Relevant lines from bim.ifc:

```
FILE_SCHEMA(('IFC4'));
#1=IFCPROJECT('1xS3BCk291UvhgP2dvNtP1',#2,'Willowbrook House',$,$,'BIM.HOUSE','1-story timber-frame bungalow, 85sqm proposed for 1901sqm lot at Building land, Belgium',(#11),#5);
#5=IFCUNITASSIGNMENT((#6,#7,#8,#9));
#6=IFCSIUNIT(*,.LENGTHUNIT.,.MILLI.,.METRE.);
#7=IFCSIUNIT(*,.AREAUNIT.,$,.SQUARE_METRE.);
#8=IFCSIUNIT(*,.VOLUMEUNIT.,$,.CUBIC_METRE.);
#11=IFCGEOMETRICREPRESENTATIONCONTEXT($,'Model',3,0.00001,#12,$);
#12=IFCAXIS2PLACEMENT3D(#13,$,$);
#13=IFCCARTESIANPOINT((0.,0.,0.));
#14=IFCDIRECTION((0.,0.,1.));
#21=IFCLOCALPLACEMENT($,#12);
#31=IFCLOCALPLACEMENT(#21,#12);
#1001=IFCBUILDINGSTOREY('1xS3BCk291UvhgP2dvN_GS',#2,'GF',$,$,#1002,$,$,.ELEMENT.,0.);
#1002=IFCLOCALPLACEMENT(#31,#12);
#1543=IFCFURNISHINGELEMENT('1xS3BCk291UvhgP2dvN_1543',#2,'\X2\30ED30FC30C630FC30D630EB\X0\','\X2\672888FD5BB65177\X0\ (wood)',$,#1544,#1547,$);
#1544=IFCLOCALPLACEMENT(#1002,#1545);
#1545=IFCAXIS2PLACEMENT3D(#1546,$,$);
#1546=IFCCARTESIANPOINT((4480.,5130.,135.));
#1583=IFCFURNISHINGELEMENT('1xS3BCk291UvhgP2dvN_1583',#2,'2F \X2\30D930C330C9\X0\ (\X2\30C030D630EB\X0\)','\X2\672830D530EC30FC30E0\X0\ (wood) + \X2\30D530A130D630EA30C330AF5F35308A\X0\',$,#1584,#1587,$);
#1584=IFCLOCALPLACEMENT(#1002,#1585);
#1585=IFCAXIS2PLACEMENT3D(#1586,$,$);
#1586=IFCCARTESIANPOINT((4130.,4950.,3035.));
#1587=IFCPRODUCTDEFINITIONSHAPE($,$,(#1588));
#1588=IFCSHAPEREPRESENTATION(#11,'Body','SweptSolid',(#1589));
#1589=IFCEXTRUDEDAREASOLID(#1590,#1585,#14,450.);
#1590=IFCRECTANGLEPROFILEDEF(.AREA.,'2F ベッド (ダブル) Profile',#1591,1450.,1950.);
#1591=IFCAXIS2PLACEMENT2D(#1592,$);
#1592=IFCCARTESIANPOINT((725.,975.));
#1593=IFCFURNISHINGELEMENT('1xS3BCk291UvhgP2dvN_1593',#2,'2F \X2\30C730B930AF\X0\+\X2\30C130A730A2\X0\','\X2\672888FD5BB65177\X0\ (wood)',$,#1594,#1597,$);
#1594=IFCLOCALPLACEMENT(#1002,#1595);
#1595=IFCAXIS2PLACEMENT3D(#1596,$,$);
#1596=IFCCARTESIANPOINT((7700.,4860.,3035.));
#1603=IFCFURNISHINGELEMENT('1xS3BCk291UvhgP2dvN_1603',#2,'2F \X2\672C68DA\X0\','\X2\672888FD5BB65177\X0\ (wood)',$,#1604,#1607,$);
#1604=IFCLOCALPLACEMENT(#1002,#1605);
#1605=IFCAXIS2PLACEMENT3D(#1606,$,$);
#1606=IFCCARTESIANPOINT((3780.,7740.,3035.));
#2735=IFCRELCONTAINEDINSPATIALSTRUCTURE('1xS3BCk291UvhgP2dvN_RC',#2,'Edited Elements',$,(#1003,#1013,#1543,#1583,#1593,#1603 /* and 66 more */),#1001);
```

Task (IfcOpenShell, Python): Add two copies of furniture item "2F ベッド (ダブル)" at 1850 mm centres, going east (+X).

```python
import numpy as np
import ifcopenshell
import ifcopenshell.api.geometry
import ifcopenshell.api.root
import ifcopenshell.util.element
import ifcopenshell.util.placement

model = ifcopenshell.open("bim.ifc")


def reuse_history(source, copy):
    """copy_class also copies each property set's owner history, people and application; keep the originals."""
    for rel in copy.IsDefinedBy:
        if rel.is_a("IfcRelDefinesByProperties") and (history := rel.RelatingPropertyDefinition.OwnerHistory):
            rel.RelatingPropertyDefinition.OwnerHistory = source.OwnerHistory
            ifcopenshell.util.element.remove_deep2(model, history)


source = model.by_guid("1xS3BCk291UvhgP2dvN_1583")
base = ifcopenshell.util.placement.get_local_placement(source.ObjectPlacement)
step = np.array([1.0, 0.0, 0.0]) * 1850.0

for i in range(1, 3):
    copy = ifcopenshell.api.root.copy_class(model, product=source)
    copy.Representation = ifcopenshell.util.element.copy_deep(
        model, source.Representation, exclude=["IfcGeometricRepresentationContext", "IfcRepresentationMap"]
    )
    reuse_history(source, copy)
    matrix = base.copy()
    matrix[:3, 3] += i * step
    print("added at", matrix[:3, 3].round(3) + 0.0)
    ifcopenshell.api.geometry.edit_object_placement(model, product=copy, matrix=matrix, is_si=False)

model.write("bim_v2.ifc")
```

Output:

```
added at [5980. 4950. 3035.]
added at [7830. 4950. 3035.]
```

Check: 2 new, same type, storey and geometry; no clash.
